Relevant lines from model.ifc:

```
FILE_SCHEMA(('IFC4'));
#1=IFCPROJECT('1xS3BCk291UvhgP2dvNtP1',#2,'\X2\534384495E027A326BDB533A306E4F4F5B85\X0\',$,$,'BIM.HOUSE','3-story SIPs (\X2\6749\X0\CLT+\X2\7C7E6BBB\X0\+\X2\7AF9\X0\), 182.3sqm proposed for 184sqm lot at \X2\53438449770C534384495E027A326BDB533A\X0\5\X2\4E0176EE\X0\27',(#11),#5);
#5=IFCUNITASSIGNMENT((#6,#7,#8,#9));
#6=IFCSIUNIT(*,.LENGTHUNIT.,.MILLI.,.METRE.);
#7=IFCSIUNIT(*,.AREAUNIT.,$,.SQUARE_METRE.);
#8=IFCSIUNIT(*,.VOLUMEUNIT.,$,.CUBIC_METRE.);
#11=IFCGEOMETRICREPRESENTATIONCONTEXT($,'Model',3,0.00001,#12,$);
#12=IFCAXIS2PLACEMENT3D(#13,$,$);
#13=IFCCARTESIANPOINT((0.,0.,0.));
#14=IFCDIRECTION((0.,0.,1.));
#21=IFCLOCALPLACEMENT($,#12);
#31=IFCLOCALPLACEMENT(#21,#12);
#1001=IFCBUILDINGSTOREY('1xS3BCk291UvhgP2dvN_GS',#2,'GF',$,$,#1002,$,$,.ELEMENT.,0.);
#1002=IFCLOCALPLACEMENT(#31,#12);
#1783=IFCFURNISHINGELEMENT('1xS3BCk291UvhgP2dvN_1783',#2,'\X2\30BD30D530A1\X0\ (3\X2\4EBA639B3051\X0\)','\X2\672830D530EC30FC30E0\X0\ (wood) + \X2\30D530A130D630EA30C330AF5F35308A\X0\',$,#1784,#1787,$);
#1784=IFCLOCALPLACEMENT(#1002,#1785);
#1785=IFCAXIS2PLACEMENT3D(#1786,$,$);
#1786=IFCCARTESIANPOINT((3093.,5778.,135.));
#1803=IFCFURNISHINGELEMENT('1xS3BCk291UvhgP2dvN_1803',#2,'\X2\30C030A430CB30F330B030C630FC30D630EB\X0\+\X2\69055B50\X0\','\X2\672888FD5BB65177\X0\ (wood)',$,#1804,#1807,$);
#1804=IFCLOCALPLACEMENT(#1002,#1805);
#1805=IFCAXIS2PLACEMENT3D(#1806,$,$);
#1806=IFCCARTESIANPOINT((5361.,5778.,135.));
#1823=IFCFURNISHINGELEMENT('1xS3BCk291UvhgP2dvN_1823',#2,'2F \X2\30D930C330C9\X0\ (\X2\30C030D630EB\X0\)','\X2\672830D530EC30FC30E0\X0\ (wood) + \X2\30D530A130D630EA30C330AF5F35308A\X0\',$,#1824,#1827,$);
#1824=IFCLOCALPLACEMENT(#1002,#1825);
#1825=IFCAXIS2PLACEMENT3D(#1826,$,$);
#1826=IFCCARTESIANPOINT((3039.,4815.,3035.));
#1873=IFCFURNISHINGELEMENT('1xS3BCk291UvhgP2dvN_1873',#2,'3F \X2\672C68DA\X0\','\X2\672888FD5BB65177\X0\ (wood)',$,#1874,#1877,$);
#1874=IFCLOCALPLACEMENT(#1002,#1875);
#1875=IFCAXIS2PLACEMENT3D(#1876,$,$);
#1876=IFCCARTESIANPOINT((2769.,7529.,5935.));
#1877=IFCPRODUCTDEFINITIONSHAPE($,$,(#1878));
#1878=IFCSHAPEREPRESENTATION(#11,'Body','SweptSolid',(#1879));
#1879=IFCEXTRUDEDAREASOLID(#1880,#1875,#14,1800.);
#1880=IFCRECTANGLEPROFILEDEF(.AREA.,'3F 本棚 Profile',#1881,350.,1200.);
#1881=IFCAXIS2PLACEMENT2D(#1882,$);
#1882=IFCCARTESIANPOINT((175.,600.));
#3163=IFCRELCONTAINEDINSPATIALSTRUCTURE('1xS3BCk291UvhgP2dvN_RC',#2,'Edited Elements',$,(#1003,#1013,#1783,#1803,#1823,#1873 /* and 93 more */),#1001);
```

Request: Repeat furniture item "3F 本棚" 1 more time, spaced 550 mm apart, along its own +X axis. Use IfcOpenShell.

```python
import ifcopenshell
import ifcopenshell.api.geometry
import ifcopenshell.api.root
import ifcopenshell.util.element
import ifcopenshell.util.placement
import ifcopenshell.util.unit

model = ifcopenshell.open("model.ifc")
unit_scale = ifcopenshell.util.unit.calculate_unit_scale(model)


def reuse_history(source, copy):
    """copy_class also copies each property set's owner history, people and application; keep the originals."""
    for rel in copy.IsDefinedBy:
        if rel.is_a("IfcRelDefinesByProperties") and (history := rel.RelatingPropertyDefinition.OwnerHistory):
            rel.RelatingPropertyDefinition.OwnerHistory = source.OwnerHistory
            ifcopenshell.util.element.remove_deep2(model, history)


source = model.by_guid("1xS3BCk291UvhgP2dvN_1873")
base = ifcopenshell.util.placement.get_local_placement(source.ObjectPlacement)
step = base[:3, 0] * 0.55 / unit_scale

for i in range(1, 2):
    copy = ifcopenshell.api.root.copy_class(model, product=source)
    copy.Representation = ifcopenshell.util.element.copy_deep(
        model, source.Representation, exclude=["IfcGeometricRepresentationContext", "IfcRepresentationMap"]
    )
    reuse_history(source, copy)
    matrix = base.copy()
    matrix[:3, 3] += i * step
    print("added at", matrix[:3, 3].round(3) + 0.0)
    ifcopenshell.api.geometry.edit_object_placement(model, product=copy, matrix=matrix, is_si=False)

model.write("model_v2.ifc")
```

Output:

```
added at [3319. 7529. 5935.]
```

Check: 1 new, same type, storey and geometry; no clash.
